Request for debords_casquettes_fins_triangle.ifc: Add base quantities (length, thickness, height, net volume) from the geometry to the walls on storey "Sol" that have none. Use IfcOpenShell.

First a look at what the model holds.

```python
import ifcopenshell
import ifcopenshell.util.element
import ifcopenshell.util.unit

model = ifcopenshell.open("debords_casquettes_fins_triangle.ifc")
print(model.schema)
for unit_type in ("LENGTHUNIT", "AREAUNIT", "VOLUMEUNIT"):
    print(unit_type, ifcopenshell.util.unit.calculate_unit_scale(model, unit_type))
storey = next(s for s in model.by_type("IfcBuildingStorey") if s.Name == "Sol")
walls = [e for e in ifcopenshell.util.element.get_decomposition(storey) if e.is_a("IfcWall")]
for e in sorted(walls, key=lambda e: e.id()):
    print(e.id(), e.is_a(), e.Name, list(ifcopenshell.util.element.get_psets(e, qtos_only=True)), sep=" | ")
```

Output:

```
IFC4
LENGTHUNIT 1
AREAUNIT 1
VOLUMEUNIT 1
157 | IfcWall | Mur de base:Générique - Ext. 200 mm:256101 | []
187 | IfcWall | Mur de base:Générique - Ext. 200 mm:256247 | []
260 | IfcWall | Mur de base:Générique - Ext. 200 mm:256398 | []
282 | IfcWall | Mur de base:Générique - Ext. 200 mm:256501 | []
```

```python
import ifcopenshell
import ifcopenshell.api.pset
import ifcopenshell.geom
import ifcopenshell.util.element
import ifcopenshell.util.shape
import ifcopenshell.util.unit

model = ifcopenshell.open("debords_casquettes_fins_triangle.ifc")
unit_scale = ifcopenshell.util.unit.calculate_unit_scale(model)
volume_scale = ifcopenshell.util.unit.calculate_unit_scale(model, "VOLUMEUNIT")
settings = ifcopenshell.geom.settings()

storey = next(s for s in model.by_type("IfcBuildingStorey") if s.Name == "Sol")
walls = [e for e in ifcopenshell.util.element.get_decomposition(storey) if e.is_a("IfcWall")]

for e in sorted(walls, key=lambda e: e.id()):
    if ifcopenshell.util.element.get_psets(e, qtos_only=True, should_inherit=False):
        continue
    # Geometry comes back in metres, in the element's own axes.
    shape = ifcopenshell.geom.create_shape(settings, e)
    values = {
        "Length": ifcopenshell.util.shape.get_x(shape.geometry) / unit_scale,
        "Width": ifcopenshell.util.shape.get_y(shape.geometry) / unit_scale,
        "Height": ifcopenshell.util.shape.get_z(shape.geometry) / unit_scale,
        "NetVolume": ifcopenshell.util.shape.get_volume(shape.geometry) / volume_scale,
    }
    qto = ifcopenshell.api.pset.add_qto(model, product=e, name="Qto_WallBaseQuantities")
    ifcopenshell.api.pset.edit_qto(model, qto=qto, properties=values)
    print(e.id(), {k: round(v, 3) for k, v in values.items()})

model.write("debords_casquettes_fins_triangle-out.ifc")
```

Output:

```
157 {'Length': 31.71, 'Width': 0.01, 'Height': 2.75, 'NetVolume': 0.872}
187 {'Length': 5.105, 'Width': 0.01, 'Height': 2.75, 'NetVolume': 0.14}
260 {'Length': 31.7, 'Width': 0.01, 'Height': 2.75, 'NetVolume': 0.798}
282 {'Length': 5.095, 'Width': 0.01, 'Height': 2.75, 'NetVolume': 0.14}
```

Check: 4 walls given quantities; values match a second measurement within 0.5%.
